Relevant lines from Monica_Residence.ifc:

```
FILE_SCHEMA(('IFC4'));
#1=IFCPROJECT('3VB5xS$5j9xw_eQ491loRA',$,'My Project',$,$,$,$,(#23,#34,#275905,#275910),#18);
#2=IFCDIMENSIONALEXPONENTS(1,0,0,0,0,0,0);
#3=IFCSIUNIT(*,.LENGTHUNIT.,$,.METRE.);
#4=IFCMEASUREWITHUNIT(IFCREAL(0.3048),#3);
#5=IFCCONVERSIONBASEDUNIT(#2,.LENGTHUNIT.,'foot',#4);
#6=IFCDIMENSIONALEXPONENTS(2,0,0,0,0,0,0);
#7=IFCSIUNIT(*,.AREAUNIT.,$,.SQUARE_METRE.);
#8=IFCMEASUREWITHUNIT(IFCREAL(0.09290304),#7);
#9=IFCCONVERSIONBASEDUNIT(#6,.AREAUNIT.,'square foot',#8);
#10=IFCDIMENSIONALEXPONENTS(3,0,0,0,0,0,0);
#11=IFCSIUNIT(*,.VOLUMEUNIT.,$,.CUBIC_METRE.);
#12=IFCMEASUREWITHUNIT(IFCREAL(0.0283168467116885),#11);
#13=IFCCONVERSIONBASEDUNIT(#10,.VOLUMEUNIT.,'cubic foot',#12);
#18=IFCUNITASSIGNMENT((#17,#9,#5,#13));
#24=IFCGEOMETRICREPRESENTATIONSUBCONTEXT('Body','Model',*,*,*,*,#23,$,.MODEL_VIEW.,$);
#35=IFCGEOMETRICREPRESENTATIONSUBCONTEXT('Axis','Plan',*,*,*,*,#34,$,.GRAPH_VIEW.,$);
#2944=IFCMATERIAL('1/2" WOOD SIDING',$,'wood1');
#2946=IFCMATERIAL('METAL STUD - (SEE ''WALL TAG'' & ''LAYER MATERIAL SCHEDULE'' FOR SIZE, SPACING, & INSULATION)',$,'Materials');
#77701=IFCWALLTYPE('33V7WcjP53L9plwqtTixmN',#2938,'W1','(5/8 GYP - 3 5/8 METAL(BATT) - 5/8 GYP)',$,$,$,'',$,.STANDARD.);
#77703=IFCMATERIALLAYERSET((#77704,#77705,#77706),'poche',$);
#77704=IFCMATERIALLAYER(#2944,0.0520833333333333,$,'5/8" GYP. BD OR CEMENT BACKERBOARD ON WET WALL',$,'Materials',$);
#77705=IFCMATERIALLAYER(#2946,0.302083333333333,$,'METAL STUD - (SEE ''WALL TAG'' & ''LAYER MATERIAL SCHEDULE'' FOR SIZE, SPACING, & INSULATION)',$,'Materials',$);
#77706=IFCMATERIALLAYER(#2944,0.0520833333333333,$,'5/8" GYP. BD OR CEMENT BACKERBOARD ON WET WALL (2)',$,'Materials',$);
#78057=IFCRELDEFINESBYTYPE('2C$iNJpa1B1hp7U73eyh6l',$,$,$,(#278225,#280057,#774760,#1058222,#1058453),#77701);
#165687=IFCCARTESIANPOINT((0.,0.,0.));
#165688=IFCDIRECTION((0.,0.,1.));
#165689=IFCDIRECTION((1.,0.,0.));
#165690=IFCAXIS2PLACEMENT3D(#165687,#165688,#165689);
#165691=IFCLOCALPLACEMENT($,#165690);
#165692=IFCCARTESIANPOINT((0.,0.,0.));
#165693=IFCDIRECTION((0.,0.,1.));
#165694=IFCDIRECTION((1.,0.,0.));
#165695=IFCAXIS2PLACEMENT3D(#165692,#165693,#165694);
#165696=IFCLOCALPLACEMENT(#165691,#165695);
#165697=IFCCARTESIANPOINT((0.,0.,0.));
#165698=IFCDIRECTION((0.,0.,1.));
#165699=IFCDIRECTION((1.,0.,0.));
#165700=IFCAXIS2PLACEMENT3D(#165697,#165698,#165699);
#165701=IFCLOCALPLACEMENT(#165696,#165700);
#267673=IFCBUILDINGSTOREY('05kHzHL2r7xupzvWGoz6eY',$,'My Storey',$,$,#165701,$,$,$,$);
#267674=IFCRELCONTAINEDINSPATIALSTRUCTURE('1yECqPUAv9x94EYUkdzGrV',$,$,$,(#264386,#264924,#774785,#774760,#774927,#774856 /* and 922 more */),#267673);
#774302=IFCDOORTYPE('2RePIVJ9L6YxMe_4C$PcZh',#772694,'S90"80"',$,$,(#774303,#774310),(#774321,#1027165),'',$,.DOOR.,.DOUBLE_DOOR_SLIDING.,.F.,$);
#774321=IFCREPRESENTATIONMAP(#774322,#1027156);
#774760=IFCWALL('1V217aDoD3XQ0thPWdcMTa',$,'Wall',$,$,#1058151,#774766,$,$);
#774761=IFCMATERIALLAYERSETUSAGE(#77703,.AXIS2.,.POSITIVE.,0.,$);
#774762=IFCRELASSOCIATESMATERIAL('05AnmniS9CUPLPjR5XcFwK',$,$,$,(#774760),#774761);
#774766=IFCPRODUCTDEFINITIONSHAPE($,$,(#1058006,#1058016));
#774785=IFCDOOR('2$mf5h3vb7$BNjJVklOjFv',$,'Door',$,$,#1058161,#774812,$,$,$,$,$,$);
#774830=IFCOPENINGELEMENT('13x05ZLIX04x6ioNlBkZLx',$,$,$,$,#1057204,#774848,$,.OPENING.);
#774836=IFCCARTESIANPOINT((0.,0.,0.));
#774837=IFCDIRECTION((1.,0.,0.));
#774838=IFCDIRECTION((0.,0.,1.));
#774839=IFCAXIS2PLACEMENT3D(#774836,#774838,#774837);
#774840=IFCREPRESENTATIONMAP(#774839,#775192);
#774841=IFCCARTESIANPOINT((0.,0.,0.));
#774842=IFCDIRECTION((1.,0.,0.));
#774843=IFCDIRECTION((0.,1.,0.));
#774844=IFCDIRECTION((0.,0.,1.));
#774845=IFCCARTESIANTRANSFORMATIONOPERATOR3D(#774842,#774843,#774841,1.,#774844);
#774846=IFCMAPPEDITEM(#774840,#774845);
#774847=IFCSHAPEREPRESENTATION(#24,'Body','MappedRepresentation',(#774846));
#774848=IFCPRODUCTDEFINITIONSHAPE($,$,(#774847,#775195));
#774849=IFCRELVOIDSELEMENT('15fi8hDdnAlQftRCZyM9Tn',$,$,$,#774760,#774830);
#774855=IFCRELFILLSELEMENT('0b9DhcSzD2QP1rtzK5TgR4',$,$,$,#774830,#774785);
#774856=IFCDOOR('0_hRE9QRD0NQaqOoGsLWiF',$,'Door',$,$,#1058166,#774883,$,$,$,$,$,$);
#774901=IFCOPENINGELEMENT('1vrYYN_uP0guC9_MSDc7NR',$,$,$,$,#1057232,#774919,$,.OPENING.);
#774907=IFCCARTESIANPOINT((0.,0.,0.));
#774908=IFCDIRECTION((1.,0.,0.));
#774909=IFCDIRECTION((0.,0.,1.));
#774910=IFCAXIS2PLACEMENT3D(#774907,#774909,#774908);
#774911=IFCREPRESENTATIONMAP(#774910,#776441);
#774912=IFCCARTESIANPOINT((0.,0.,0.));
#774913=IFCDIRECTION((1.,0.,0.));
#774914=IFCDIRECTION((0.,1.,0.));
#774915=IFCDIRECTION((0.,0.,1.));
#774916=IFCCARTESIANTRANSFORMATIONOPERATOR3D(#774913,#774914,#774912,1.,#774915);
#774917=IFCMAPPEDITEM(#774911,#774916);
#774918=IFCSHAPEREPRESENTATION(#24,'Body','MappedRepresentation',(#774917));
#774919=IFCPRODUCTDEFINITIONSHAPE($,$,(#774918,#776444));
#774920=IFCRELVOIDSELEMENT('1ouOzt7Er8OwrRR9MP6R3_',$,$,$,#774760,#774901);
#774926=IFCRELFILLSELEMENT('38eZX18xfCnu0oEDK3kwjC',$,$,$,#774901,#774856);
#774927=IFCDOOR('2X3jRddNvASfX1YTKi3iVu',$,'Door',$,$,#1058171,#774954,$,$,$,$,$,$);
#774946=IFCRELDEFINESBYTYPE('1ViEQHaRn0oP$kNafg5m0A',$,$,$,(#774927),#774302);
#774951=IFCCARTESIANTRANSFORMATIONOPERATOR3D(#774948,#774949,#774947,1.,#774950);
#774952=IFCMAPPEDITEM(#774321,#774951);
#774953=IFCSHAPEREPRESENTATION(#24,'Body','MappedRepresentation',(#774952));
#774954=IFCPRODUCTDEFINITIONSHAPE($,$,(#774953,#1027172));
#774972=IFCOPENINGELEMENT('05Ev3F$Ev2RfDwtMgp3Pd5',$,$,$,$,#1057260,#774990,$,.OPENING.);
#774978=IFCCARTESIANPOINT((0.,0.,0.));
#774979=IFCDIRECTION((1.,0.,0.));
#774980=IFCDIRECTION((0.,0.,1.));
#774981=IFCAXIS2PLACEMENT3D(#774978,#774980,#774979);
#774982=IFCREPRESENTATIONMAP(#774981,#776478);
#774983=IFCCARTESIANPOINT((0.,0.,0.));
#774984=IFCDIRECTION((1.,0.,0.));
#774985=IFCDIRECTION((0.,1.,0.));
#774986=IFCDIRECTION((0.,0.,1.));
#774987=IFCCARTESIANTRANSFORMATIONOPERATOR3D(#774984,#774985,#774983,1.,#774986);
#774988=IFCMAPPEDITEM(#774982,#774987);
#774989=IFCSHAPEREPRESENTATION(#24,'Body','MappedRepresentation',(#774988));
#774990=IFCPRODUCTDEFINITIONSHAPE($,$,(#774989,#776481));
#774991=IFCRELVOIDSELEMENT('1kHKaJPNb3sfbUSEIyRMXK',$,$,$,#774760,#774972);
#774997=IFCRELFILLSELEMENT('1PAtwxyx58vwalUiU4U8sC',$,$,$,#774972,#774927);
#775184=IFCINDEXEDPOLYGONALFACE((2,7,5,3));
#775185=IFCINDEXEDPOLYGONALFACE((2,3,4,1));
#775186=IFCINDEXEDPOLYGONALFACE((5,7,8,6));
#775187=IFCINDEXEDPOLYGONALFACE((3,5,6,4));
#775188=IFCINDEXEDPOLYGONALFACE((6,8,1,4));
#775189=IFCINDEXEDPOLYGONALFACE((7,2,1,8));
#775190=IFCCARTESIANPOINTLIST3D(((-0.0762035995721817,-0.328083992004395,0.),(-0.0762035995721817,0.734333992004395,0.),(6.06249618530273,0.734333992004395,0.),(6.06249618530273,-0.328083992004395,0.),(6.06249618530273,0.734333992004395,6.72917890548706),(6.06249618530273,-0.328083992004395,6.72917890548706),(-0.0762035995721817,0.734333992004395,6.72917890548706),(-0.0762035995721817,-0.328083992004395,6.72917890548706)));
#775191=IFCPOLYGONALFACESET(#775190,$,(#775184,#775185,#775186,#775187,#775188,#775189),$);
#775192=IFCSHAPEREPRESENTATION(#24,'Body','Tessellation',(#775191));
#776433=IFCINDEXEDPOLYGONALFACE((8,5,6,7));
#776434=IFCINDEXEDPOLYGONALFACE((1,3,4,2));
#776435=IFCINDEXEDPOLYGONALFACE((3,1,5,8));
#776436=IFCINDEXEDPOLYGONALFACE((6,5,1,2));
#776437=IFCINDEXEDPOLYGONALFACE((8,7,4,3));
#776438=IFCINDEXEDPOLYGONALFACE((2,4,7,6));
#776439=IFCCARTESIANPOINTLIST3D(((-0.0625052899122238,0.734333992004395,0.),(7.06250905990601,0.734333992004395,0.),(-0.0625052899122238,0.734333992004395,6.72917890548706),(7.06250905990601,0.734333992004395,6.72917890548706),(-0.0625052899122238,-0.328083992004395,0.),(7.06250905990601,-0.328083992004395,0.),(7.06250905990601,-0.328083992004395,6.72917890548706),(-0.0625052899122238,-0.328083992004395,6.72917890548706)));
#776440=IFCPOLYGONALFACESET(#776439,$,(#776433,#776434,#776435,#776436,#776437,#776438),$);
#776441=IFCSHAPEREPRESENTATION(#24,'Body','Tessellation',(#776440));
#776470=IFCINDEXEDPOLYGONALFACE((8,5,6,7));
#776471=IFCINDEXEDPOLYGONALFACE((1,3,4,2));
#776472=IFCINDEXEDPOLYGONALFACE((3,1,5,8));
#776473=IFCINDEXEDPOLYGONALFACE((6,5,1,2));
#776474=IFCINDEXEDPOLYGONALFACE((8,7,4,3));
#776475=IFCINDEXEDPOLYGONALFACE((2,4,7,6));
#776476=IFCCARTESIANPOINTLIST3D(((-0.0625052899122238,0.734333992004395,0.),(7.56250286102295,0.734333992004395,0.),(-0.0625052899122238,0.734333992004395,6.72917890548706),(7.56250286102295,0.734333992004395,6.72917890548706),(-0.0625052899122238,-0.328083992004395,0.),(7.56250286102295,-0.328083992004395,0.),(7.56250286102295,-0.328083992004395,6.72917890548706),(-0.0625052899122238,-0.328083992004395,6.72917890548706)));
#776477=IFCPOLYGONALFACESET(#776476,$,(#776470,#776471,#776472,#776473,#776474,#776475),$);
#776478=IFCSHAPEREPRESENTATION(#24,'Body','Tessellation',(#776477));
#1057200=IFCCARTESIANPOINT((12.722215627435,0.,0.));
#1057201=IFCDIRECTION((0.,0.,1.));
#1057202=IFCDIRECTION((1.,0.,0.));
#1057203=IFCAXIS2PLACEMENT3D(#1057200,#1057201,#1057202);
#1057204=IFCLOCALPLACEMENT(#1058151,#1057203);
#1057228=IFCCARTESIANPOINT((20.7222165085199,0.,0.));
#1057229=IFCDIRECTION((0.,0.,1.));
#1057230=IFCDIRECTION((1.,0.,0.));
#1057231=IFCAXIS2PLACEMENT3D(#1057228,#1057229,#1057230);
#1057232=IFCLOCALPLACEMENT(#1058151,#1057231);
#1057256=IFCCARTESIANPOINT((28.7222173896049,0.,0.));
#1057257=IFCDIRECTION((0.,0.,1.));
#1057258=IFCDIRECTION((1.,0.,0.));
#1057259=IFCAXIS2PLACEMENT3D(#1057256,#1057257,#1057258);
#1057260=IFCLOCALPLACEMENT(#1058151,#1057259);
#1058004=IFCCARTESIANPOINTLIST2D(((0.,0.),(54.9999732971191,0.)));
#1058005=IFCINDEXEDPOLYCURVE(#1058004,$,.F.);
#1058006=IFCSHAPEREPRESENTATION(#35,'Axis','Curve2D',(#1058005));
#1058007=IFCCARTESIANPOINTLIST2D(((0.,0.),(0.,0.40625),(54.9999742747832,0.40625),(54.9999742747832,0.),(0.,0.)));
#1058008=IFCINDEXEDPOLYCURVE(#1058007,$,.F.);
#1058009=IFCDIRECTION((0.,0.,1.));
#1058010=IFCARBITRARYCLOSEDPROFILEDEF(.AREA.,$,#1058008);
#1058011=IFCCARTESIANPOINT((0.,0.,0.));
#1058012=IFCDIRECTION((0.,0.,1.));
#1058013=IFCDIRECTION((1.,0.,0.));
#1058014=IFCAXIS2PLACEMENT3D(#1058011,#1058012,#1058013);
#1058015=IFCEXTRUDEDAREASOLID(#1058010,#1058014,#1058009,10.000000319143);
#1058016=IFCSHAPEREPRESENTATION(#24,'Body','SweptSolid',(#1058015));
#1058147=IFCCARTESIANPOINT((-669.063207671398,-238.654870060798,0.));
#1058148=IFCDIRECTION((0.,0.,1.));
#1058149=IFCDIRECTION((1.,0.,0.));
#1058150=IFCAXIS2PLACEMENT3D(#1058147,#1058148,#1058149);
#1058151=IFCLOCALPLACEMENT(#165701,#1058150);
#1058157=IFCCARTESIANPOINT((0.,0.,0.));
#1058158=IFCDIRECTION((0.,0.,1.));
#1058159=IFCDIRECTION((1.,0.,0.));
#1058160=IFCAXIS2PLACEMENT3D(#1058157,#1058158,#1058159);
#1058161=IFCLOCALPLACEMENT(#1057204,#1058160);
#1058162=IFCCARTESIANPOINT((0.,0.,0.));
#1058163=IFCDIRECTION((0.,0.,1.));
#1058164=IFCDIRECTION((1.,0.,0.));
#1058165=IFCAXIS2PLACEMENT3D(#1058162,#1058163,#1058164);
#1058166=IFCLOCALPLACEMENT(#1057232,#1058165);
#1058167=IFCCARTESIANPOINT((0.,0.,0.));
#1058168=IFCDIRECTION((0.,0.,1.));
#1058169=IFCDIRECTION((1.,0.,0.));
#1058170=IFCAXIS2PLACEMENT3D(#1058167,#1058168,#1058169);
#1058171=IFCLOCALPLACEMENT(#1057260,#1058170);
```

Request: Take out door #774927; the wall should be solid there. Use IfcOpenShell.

```python
import ifcopenshell
import ifcopenshell.api.feature
import ifcopenshell.api.root
import ifcopenshell.geom
import ifcopenshell.util.shape

model = ifcopenshell.open("Monica_Residence.ifc")
settings = ifcopenshell.geom.settings()


def volume(element):
    """Net volume in cubic metres, openings subtracted."""
    shape = ifcopenshell.geom.create_shape(settings, element)
    return ifcopenshell.util.shape.get_volume(shape.geometry)


door = model.by_id(774927)
opening = door.FillsVoids[0].RelatingOpeningElement
wall = opening.VoidsElements[0].RelatingBuildingElement
before = volume(wall)

ifcopenshell.api.root.remove_product(model, product=door)
ifcopenshell.api.feature.remove_feature(model, feature=opening)

after = volume(wall)

print(f"wall volume {before:.3f} -> {after:.3f} m3")

model.write("Monica_Residence_edited.ifc")
```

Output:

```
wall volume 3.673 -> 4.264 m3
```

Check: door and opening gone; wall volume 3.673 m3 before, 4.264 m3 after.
